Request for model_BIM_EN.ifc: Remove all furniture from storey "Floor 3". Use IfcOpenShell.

First a look at what the model holds.

```python
import ifcopenshell
import ifcopenshell.util.element

model = ifcopenshell.open("model_BIM_EN.ifc")
print(model.schema)
storey = next(s for s in model.by_type("IfcBuildingStorey") if s.Name == "Floor 3")
furniture = [e for e in ifcopenshell.util.element.get_decomposition(storey) if e.is_a("IfcFurnishingElement")]
seen = {}
for e in furniture:
    element_type = ifcopenshell.util.element.get_type(e)
    name = element_type.Name if element_type not in (None, e) else None
    seen[name] = seen.get(name, 0) + 1
for name, count in sorted(seen.items(), key=str):
    print(count, "x", name)
```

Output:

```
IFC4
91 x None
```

```python
import ifcopenshell
import ifcopenshell.api.root
import ifcopenshell.util.element

model = ifcopenshell.open("model_BIM_EN.ifc")

storey = next(s for s in model.by_type("IfcBuildingStorey") if s.Name == "Floor 3")
furniture = [e for e in ifcopenshell.util.element.get_decomposition(storey) if e.is_a("IfcFurnishingElement")]

for e in furniture:
    ifcopenshell.api.root.remove_product(model, product=e)
print(len(furniture), "removed")

model.write("model_BIM_EN_v2.ifc")
```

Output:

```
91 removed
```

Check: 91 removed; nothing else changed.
